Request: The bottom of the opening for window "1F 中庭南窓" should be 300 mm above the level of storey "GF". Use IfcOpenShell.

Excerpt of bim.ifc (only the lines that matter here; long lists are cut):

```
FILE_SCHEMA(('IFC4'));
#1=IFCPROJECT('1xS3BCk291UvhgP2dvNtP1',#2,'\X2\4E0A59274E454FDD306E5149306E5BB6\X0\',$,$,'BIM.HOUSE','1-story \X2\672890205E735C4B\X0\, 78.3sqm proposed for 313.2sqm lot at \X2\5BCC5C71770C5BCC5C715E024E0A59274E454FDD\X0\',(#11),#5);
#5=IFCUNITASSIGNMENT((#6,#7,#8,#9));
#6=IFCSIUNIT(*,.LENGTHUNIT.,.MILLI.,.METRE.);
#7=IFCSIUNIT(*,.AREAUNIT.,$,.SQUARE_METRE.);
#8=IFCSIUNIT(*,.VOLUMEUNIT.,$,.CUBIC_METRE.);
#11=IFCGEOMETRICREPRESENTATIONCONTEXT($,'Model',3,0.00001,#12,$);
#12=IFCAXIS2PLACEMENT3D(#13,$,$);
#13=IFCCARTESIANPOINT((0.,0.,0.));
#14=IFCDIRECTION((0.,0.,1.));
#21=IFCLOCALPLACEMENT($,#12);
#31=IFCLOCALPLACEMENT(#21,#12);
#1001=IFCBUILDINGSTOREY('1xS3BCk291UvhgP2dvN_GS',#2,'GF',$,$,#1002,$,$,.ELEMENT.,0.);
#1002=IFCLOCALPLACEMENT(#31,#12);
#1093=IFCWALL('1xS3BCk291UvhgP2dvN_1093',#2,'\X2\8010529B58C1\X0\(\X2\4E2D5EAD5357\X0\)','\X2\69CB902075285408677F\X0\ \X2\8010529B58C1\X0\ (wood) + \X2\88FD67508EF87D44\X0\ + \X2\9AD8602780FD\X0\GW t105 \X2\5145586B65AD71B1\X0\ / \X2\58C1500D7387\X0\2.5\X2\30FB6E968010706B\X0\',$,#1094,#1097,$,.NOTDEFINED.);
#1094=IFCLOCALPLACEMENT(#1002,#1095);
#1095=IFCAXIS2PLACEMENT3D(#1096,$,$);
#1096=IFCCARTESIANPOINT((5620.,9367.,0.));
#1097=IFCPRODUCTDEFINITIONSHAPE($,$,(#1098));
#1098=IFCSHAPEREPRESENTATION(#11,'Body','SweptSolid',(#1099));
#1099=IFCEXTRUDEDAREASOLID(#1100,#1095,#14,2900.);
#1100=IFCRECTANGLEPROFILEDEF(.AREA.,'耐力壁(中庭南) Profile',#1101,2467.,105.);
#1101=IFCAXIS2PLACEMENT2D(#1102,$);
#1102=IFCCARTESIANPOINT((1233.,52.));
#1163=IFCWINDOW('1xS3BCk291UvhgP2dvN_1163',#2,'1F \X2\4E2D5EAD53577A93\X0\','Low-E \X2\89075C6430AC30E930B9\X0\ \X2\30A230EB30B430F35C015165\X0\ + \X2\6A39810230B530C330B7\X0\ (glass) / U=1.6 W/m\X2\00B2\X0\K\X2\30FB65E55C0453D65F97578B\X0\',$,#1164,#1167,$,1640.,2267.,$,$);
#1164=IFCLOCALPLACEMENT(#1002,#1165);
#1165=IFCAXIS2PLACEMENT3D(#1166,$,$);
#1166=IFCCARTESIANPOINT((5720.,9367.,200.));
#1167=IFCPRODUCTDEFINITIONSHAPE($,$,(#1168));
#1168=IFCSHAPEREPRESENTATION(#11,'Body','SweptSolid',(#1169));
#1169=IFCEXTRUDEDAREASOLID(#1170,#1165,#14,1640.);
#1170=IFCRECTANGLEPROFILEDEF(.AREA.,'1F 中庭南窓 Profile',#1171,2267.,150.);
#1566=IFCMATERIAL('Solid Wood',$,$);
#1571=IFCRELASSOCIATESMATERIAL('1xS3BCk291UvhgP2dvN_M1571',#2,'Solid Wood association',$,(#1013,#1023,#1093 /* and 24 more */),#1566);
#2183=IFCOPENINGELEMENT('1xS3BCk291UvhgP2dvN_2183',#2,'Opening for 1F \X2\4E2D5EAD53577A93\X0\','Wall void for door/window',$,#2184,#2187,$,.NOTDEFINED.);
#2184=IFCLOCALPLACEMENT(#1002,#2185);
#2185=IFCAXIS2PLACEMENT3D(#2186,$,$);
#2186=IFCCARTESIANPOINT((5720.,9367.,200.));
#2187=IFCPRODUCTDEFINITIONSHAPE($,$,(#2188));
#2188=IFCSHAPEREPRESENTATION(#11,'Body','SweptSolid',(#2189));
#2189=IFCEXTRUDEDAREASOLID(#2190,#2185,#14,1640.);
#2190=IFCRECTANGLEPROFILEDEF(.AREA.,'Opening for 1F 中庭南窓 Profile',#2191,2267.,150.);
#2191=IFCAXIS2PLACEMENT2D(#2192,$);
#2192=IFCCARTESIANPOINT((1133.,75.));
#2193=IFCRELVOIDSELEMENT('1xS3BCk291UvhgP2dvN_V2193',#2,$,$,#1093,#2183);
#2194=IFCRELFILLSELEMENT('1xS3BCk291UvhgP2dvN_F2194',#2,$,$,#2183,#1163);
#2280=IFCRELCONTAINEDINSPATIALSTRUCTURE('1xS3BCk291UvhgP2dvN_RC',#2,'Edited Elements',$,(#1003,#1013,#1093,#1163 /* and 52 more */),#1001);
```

```python
import numpy as np
import ifcopenshell
import ifcopenshell.api.geometry
import ifcopenshell.geom
import ifcopenshell.util.element
import ifcopenshell.util.placement
import ifcopenshell.util.shape
import ifcopenshell.util.unit

model = ifcopenshell.open("bim.ifc")
unit_scale = ifcopenshell.util.unit.calculate_unit_scale(model)

window = model.by_guid("1xS3BCk291UvhgP2dvN_1163")
opening = window.FillsVoids[0].RelatingOpeningElement
storey = ifcopenshell.util.element.get_container(window, ifc_class="IfcBuildingStorey")
level = ifcopenshell.util.placement.get_local_placement(storey.ObjectPlacement)[2, 3]

# The opening's origin need not be at the sill, so measure its lowest point.
shape = ifcopenshell.geom.create_shape(ifcopenshell.geom.settings(), opening)
bottom = ifcopenshell.util.shape.get_shape_bottom_elevation(shape, shape.geometry) / unit_scale
dz = level + 0.3 / unit_scale - bottom

shift = np.array([0.0, 0.0, dz])
# The window is not placed relative to its opening, so move both.
for product in (opening, window):
    matrix = ifcopenshell.util.placement.get_local_placement(product.ObjectPlacement)
    matrix[:3, 3] += shift
    ifcopenshell.api.geometry.edit_object_placement(model, product=product, matrix=matrix, is_si=False)

print(f"moved by {dz * unit_scale:+.3f} m")

model.write("bim-out.ifc")
```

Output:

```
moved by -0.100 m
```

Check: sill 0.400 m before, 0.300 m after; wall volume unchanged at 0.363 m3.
